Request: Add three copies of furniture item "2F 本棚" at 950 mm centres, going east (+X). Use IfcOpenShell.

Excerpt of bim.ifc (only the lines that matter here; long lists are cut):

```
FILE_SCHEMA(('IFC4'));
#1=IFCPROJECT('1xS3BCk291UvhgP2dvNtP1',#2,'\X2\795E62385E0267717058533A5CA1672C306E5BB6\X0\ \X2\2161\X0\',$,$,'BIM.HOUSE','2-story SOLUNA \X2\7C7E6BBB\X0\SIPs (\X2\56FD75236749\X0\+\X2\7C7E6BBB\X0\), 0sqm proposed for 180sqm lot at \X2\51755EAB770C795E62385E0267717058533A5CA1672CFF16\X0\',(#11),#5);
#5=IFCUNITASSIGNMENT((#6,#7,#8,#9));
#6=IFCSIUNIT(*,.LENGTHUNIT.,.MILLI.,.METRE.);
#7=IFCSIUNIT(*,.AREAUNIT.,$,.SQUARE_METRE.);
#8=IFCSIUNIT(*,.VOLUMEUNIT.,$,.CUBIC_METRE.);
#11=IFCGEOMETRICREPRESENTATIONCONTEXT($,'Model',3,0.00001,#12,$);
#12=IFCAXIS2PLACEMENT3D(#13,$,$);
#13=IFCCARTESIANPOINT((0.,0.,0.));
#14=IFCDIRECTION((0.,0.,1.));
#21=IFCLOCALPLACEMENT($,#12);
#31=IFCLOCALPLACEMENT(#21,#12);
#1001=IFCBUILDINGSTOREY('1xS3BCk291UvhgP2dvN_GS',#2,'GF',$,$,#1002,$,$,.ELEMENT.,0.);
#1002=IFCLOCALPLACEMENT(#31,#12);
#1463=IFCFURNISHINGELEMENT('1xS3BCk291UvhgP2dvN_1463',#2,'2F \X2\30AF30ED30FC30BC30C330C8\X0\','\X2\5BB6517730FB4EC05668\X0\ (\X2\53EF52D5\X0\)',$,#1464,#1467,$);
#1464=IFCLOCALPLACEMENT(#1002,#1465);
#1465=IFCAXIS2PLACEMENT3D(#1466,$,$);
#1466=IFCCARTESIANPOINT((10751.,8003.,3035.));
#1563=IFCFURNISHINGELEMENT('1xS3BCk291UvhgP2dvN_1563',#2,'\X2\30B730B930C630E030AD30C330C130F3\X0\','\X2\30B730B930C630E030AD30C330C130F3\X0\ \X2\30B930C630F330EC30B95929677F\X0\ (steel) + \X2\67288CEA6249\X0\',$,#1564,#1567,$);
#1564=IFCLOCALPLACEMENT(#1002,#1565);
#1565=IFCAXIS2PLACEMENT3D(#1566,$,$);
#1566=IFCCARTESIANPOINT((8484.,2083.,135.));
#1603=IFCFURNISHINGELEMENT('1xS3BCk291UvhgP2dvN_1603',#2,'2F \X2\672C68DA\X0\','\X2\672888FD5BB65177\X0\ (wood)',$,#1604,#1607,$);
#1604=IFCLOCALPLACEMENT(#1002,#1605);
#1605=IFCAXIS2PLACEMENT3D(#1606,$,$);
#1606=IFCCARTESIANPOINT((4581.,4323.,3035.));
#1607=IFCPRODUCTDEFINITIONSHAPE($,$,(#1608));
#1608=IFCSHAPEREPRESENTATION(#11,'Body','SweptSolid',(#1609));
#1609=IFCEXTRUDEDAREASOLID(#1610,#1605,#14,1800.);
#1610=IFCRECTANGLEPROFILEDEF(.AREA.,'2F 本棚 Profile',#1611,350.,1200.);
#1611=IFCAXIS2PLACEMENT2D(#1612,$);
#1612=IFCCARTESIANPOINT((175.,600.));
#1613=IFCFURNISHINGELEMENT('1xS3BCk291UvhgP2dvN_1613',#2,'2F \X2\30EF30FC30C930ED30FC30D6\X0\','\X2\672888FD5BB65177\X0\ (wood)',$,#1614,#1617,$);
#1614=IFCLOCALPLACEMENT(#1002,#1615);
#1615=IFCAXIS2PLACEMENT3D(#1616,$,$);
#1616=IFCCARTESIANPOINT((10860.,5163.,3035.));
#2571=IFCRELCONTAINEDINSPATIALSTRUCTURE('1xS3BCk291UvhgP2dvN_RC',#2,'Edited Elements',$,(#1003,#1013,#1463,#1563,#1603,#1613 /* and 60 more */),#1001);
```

```python
import numpy as np
import ifcopenshell
import ifcopenshell.api.geometry
import ifcopenshell.api.root
import ifcopenshell.util.element
import ifcopenshell.util.placement

model = ifcopenshell.open("bim.ifc")


def reuse_history(source, copy):
    """copy_class also copies each property set's owner history, people and application; keep the originals."""
    for rel in copy.IsDefinedBy:
        if rel.is_a("IfcRelDefinesByProperties") and (history := rel.RelatingPropertyDefinition.OwnerHistory):
            rel.RelatingPropertyDefinition.OwnerHistory = source.OwnerHistory
            ifcopenshell.util.element.remove_deep2(model, history)


source = model.by_id(1603)
base = ifcopenshell.util.placement.get_local_placement(source.ObjectPlacement)
step = np.array([1.0, 0.0, 0.0]) * 950.0

for i in range(1, 4):
    copy = ifcopenshell.api.root.copy_class(model, product=source)
    copy.Representation = ifcopenshell.util.element.copy_deep(
        model, source.Representation, exclude=["IfcGeometricRepresentationContext", "IfcRepresentationMap"]
    )
    reuse_history(source, copy)
    matrix = base.copy()
    matrix[:3, 3] += i * step
    print("added at", matrix[:3, 3].round(3) + 0.0)
    ifcopenshell.api.geometry.edit_object_placement(model, product=copy, matrix=matrix, is_si=False)

model.write("bim_rev.ifc")
```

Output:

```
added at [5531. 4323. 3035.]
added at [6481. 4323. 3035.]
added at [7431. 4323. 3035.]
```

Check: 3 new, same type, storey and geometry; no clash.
